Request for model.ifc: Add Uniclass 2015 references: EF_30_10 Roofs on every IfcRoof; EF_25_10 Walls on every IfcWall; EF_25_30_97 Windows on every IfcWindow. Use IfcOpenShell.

First a look at what the model holds.

```python
import ifcopenshell

model = ifcopenshell.open("model.ifc")
print(model.schema)
print("classifications:", [c.Name for c in model.by_type("IfcClassification")])
for ifc_class in ("IfcDoor", "IfcRoof", "IfcStair", "IfcWall", "IfcWindow"):
    print(ifc_class, len(model.by_type(ifc_class)))
```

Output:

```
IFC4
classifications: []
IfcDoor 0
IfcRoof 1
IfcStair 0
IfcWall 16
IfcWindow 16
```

```python
import ifcopenshell
import ifcopenshell.api.classification

model = ifcopenshell.open("model.ifc")

system = ifcopenshell.api.classification.add_classification(model, classification="Uniclass 2015")

codes = {
    "IfcRoof": ("EF_30_10", "Roofs"),
    "IfcWall": ("EF_25_10", "Walls"),
    "IfcWindow": ("EF_25_30_97", "Windows"),
}
for ifc_class, (code, name) in codes.items():
    products = model.by_type(ifc_class)
    ifcopenshell.api.classification.add_reference(
        model, products=products, classification=system, identification=code, name=name
    )
    print(code, len(products))

model.write("model-out.ifc")
```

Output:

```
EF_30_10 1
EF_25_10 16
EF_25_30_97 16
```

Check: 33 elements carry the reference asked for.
